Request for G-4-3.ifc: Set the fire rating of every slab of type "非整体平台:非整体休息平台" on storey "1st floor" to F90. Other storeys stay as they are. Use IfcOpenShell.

First a look at what the model holds.

```python
import ifcopenshell
import ifcopenshell.util.element

model = ifcopenshell.open("G-4-3.ifc")
print(model.schema)
storey = next(s for s in model.by_type("IfcBuildingStorey") if s.Name == "1st floor")
slabs = [e for e in ifcopenshell.util.element.get_decomposition(storey) if e.is_a("IfcSlab")]
seen = {}
for e in slabs:
    element_type = ifcopenshell.util.element.get_type(e)
    key = (element_type.Name if element_type != e and element_type else None, ifcopenshell.util.element.get_pset(e, "Pset_SlabCommon", "FireRating"))
    seen[key] = seen.get(key, 0) + 1
for (name, value), count in sorted(seen.items(), key=str):
    print(count, "x", name, "|", value)
```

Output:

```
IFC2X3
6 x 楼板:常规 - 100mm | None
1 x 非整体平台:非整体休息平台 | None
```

```python
import ifcopenshell
import ifcopenshell.api.pset
import ifcopenshell.util.element

model = ifcopenshell.open("G-4-3.ifc")

storey = next(s for s in model.by_type("IfcBuildingStorey") if s.Name == "1st floor")
slabs = [e for e in ifcopenshell.util.element.get_decomposition(storey) if e.is_a("IfcSlab")]

count = 0
for e in slabs:
    element_type = ifcopenshell.util.element.get_type(e)
    if element_type in (None, e) or element_type.Name != "非整体平台:非整体休息平台":
        continue
    # add_pset returns the element's existing set when there is one.
    pset = ifcopenshell.api.pset.add_pset(model, product=e, name="Pset_SlabCommon")
    ifcopenshell.api.pset.edit_pset(model, pset=pset, properties={"FireRating": "F90"})
    count += 1

print(count, "slabs updated")

model.write("G-4-3_edited.ifc")
```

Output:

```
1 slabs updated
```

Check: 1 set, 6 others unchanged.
